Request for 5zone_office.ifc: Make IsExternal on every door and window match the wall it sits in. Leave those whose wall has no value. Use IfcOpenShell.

First a look at what the model holds.

```python
import ifcopenshell
import ifcopenshell.util.element

model = ifcopenshell.open("5zone_office.ifc")
print(model.schema)
seen = {}
for e in model.by_type("IfcDoor") + model.by_type("IfcWindow"):
    if not e.FillsVoids:
        continue
    host = e.FillsVoids[0].RelatingOpeningElement.VoidsElements[0].RelatingBuildingElement
    own = ifcopenshell.util.element.get_pset(e, f"Pset_{e.is_a()[3:].removesuffix('StandardCase')}Common", "IsExternal")
    wall = ifcopenshell.util.element.get_pset(host, "Pset_WallCommon", "IsExternal")
    seen[e.is_a(), own, wall] = seen.get((e.is_a(), own, wall), 0) + 1
for (cls, own, wall), count in sorted(seen.items(), key=str):
    print(count, cls, "IsExternal:", own, "| host wall:", wall)
```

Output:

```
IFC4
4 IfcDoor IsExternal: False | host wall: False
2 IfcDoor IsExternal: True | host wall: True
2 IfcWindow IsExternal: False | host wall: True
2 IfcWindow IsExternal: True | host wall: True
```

```python
import ifcopenshell
import ifcopenshell.api.pset
import ifcopenshell.util.element

model = ifcopenshell.open("5zone_office.ifc")

count = 0
for ifc_class, pset_name in (("IfcDoor", "Pset_DoorCommon"), ("IfcWindow", "Pset_WindowCommon")):
    for e in model.by_type(ifc_class):
        if not e.FillsVoids:
            continue
        host = e.FillsVoids[0].RelatingOpeningElement.VoidsElements[0].RelatingBuildingElement
        external = ifcopenshell.util.element.get_pset(host, "Pset_WallCommon", "IsExternal")
        if external is None or ifcopenshell.util.element.get_pset(e, pset_name, "IsExternal") == external:
            continue
        pset = ifcopenshell.api.pset.add_pset(model, product=e, name=pset_name)
        ifcopenshell.api.pset.edit_pset(model, pset=pset, properties={"IsExternal": external})
        count += 1

print(count, "updated")

model.write("5zone_office_v2.ifc")
```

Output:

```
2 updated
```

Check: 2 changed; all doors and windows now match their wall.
